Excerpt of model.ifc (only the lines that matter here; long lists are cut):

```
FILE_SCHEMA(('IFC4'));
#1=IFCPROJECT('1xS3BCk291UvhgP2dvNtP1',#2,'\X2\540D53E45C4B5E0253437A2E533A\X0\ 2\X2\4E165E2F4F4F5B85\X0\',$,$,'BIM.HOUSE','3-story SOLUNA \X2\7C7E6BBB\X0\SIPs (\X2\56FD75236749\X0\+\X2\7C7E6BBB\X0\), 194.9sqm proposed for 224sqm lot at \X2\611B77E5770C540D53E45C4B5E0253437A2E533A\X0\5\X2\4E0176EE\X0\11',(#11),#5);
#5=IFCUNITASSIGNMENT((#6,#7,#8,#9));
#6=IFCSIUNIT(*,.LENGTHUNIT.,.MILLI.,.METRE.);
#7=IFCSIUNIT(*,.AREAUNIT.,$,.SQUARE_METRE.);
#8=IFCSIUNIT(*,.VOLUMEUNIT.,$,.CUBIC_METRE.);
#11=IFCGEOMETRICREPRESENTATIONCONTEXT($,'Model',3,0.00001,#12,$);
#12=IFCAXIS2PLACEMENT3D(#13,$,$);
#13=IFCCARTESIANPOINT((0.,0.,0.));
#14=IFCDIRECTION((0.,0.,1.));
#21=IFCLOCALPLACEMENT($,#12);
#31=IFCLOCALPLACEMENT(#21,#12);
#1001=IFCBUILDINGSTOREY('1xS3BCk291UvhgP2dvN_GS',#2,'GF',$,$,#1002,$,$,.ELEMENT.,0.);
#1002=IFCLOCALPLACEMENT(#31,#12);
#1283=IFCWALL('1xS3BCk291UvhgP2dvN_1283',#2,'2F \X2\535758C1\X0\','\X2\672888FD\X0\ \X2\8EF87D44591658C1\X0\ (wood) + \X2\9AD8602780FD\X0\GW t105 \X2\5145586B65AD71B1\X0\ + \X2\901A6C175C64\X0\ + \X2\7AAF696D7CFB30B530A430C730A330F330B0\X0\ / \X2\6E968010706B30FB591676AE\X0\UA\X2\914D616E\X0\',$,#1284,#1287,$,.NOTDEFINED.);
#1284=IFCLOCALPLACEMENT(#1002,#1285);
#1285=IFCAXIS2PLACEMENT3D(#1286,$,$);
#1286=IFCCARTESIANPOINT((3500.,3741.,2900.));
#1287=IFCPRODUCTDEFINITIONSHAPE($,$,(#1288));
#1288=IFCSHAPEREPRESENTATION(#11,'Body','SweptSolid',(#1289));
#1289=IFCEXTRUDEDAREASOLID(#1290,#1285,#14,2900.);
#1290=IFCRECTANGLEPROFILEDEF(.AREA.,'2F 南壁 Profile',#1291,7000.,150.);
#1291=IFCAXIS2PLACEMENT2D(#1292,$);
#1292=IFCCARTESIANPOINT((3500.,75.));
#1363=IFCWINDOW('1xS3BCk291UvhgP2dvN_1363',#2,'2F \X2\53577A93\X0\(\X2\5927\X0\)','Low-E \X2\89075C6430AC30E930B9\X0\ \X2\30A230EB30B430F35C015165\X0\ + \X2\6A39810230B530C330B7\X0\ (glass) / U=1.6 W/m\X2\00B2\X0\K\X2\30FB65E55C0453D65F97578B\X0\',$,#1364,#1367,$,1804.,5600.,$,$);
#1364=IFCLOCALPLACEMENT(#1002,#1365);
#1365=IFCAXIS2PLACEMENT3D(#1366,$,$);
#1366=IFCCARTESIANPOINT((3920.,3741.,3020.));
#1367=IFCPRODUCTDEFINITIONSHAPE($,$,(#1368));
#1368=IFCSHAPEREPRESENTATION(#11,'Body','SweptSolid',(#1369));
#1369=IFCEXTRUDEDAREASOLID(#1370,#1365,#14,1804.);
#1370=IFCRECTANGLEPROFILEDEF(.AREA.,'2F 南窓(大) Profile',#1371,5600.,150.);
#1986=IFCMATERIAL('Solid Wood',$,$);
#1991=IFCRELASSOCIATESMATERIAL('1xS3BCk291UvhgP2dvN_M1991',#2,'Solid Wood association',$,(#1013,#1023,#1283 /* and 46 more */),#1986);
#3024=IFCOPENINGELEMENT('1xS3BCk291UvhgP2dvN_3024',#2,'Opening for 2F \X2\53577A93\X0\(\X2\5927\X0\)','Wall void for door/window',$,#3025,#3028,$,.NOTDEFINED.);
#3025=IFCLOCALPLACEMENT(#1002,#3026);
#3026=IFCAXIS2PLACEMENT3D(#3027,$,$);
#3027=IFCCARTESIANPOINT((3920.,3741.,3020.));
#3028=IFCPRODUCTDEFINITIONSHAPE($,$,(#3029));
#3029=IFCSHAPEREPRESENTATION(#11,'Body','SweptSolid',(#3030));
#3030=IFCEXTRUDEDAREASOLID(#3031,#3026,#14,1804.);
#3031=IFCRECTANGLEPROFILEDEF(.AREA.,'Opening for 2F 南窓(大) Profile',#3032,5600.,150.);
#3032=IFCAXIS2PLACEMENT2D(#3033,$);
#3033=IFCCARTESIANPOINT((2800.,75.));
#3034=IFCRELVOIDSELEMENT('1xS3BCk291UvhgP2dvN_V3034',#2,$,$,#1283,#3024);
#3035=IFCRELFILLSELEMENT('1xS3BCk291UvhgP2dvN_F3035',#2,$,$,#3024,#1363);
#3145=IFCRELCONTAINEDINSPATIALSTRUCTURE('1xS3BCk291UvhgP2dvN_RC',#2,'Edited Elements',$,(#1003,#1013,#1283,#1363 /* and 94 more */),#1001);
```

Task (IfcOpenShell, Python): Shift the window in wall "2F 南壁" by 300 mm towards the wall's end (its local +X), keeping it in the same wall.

```python
import ifcopenshell
import ifcopenshell.api.geometry
import ifcopenshell.util.placement
import ifcopenshell.util.unit

model = ifcopenshell.open("model.ifc")
unit_scale = ifcopenshell.util.unit.calculate_unit_scale(model)

window = model.by_guid("1xS3BCk291UvhgP2dvN_1363")
opening = window.FillsVoids[0].RelatingOpeningElement
wall = opening.VoidsElements[0].RelatingBuildingElement

wall_matrix = ifcopenshell.util.placement.get_local_placement(wall.ObjectPlacement)
shift = wall_matrix[:3, 0] * 0.3 / unit_scale
before = ifcopenshell.util.placement.get_local_placement(window.ObjectPlacement)[:3, 3].copy()

# The window is not placed relative to its opening, so move both.
for product in (opening, window):
    matrix = ifcopenshell.util.placement.get_local_placement(product.ObjectPlacement)
    matrix[:3, 3] += shift
    ifcopenshell.api.geometry.edit_object_placement(model, product=product, matrix=matrix, is_si=False)

after = ifcopenshell.util.placement.get_local_placement(window.ObjectPlacement)[:3, 3]
print("window moved by", (after - before).round(3) + 0.0)

model.write("model_rev.ifc")
```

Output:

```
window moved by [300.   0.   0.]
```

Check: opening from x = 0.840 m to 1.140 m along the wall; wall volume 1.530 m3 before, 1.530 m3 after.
